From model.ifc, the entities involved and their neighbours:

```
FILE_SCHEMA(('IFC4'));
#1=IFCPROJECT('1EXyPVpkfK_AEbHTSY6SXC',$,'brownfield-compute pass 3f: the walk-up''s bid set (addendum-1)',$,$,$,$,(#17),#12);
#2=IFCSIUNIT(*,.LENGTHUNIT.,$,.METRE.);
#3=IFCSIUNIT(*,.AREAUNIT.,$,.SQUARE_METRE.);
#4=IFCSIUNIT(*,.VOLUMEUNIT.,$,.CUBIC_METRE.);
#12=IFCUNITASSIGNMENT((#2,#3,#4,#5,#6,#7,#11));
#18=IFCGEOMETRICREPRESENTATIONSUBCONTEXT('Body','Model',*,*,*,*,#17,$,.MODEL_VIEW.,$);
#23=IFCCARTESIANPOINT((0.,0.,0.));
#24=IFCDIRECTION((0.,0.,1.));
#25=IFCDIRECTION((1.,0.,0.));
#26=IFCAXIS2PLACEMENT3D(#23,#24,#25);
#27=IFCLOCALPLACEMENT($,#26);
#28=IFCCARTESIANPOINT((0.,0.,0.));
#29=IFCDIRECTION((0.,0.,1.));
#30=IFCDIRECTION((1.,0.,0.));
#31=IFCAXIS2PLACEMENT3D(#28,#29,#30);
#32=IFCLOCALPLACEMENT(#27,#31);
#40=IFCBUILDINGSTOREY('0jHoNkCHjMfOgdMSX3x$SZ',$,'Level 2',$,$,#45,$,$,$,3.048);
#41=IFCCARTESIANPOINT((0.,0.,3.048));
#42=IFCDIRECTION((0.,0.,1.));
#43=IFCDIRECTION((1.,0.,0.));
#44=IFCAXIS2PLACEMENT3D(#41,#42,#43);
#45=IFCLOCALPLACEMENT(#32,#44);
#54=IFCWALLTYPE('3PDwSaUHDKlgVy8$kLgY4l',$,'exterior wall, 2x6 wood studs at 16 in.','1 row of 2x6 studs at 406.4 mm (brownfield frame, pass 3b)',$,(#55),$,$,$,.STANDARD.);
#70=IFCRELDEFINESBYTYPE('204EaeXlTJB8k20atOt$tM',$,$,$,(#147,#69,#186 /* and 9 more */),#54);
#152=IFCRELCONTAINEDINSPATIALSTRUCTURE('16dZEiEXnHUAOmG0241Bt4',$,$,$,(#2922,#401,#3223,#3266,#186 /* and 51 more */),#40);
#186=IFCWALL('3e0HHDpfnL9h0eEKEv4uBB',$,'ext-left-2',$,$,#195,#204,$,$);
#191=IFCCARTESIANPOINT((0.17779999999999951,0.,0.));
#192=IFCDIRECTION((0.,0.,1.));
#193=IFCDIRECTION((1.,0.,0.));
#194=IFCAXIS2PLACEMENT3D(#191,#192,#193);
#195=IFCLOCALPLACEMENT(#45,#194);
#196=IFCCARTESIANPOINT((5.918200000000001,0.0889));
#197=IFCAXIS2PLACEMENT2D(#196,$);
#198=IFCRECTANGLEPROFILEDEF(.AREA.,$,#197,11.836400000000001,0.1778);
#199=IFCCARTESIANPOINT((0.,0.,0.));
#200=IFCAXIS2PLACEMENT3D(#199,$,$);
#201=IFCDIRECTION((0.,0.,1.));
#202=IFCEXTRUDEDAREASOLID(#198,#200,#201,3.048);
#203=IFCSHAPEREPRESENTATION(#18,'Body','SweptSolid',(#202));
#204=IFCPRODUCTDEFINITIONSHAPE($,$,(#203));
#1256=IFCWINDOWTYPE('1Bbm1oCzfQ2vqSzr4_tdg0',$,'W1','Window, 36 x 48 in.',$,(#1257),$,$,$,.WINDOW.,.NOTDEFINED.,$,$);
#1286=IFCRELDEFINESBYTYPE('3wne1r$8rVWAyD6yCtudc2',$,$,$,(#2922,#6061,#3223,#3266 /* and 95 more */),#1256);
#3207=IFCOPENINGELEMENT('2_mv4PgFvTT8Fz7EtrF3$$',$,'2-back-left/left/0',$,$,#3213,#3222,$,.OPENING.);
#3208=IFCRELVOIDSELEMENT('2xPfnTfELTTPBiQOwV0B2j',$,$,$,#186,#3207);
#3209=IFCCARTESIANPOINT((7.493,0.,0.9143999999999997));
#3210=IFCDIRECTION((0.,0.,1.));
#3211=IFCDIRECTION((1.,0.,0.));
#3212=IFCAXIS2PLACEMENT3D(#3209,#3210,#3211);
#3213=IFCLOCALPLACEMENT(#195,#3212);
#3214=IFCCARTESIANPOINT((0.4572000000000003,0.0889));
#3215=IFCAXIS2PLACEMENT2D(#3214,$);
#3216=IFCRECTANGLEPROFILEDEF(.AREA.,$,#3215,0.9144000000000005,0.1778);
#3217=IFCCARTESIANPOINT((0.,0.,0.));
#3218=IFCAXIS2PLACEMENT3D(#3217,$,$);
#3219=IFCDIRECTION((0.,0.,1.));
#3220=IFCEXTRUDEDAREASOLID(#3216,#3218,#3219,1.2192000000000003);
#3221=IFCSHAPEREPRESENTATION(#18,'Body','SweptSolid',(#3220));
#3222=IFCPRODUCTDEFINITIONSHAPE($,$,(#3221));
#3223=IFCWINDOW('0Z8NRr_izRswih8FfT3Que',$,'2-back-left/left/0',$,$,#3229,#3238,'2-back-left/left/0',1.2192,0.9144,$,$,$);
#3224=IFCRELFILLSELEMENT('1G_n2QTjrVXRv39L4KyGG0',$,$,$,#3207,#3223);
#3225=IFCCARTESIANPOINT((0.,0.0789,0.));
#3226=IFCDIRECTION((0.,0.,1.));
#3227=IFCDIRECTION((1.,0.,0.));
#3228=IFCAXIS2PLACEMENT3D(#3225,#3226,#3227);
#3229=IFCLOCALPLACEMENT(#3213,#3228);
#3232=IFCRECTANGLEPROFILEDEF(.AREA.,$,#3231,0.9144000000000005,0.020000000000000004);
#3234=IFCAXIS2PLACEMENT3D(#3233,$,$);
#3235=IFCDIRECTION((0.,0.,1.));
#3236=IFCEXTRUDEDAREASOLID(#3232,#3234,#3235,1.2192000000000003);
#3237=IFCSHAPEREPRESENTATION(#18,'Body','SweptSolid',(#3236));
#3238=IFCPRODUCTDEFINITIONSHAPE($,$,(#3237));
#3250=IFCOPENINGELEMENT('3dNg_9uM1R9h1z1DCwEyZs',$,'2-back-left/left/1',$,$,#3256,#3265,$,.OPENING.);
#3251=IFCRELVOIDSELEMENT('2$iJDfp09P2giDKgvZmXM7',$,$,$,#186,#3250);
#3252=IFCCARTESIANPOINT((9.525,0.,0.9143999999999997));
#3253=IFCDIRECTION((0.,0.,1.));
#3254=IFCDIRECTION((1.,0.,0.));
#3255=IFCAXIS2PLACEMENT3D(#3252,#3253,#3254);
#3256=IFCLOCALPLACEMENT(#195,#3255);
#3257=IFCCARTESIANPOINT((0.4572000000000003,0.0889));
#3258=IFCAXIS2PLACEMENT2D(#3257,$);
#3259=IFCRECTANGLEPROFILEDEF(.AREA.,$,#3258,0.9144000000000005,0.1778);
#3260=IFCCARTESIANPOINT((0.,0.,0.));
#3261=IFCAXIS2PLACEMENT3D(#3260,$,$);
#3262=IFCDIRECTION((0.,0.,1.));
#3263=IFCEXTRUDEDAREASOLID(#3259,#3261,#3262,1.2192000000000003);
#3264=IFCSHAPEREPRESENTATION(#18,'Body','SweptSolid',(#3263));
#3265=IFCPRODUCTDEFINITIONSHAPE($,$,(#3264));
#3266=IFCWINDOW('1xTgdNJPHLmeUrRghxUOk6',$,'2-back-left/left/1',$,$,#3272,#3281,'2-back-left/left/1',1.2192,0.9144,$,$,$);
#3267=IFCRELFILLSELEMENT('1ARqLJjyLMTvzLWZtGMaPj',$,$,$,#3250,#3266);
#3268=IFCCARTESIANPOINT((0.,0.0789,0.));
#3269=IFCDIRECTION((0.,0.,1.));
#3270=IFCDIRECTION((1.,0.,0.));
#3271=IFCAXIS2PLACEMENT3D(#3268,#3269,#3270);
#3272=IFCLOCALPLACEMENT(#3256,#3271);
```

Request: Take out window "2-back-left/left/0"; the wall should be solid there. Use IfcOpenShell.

```python
import ifcopenshell
import ifcopenshell.api.feature
import ifcopenshell.api.root
import ifcopenshell.geom
import ifcopenshell.util.shape

model = ifcopenshell.open("model.ifc")
settings = ifcopenshell.geom.settings()


def volume(element):
    """Net volume in cubic metres, openings subtracted."""
    shape = ifcopenshell.geom.create_shape(settings, element)
    return ifcopenshell.util.shape.get_volume(shape.geometry)


window = model.by_guid("0Z8NRr_izRswih8FfT3Que")
opening = window.FillsVoids[0].RelatingOpeningElement
wall = opening.VoidsElements[0].RelatingBuildingElement
before = volume(wall)

ifcopenshell.api.root.remove_product(model, product=window)
ifcopenshell.api.feature.remove_feature(model, feature=opening)

after = volume(wall)

print(f"wall volume {before:.3f} -> {after:.3f} m3")

model.write("model_rev.ifc")
```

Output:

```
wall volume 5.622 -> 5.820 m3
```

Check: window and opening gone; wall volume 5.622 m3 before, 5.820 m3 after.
